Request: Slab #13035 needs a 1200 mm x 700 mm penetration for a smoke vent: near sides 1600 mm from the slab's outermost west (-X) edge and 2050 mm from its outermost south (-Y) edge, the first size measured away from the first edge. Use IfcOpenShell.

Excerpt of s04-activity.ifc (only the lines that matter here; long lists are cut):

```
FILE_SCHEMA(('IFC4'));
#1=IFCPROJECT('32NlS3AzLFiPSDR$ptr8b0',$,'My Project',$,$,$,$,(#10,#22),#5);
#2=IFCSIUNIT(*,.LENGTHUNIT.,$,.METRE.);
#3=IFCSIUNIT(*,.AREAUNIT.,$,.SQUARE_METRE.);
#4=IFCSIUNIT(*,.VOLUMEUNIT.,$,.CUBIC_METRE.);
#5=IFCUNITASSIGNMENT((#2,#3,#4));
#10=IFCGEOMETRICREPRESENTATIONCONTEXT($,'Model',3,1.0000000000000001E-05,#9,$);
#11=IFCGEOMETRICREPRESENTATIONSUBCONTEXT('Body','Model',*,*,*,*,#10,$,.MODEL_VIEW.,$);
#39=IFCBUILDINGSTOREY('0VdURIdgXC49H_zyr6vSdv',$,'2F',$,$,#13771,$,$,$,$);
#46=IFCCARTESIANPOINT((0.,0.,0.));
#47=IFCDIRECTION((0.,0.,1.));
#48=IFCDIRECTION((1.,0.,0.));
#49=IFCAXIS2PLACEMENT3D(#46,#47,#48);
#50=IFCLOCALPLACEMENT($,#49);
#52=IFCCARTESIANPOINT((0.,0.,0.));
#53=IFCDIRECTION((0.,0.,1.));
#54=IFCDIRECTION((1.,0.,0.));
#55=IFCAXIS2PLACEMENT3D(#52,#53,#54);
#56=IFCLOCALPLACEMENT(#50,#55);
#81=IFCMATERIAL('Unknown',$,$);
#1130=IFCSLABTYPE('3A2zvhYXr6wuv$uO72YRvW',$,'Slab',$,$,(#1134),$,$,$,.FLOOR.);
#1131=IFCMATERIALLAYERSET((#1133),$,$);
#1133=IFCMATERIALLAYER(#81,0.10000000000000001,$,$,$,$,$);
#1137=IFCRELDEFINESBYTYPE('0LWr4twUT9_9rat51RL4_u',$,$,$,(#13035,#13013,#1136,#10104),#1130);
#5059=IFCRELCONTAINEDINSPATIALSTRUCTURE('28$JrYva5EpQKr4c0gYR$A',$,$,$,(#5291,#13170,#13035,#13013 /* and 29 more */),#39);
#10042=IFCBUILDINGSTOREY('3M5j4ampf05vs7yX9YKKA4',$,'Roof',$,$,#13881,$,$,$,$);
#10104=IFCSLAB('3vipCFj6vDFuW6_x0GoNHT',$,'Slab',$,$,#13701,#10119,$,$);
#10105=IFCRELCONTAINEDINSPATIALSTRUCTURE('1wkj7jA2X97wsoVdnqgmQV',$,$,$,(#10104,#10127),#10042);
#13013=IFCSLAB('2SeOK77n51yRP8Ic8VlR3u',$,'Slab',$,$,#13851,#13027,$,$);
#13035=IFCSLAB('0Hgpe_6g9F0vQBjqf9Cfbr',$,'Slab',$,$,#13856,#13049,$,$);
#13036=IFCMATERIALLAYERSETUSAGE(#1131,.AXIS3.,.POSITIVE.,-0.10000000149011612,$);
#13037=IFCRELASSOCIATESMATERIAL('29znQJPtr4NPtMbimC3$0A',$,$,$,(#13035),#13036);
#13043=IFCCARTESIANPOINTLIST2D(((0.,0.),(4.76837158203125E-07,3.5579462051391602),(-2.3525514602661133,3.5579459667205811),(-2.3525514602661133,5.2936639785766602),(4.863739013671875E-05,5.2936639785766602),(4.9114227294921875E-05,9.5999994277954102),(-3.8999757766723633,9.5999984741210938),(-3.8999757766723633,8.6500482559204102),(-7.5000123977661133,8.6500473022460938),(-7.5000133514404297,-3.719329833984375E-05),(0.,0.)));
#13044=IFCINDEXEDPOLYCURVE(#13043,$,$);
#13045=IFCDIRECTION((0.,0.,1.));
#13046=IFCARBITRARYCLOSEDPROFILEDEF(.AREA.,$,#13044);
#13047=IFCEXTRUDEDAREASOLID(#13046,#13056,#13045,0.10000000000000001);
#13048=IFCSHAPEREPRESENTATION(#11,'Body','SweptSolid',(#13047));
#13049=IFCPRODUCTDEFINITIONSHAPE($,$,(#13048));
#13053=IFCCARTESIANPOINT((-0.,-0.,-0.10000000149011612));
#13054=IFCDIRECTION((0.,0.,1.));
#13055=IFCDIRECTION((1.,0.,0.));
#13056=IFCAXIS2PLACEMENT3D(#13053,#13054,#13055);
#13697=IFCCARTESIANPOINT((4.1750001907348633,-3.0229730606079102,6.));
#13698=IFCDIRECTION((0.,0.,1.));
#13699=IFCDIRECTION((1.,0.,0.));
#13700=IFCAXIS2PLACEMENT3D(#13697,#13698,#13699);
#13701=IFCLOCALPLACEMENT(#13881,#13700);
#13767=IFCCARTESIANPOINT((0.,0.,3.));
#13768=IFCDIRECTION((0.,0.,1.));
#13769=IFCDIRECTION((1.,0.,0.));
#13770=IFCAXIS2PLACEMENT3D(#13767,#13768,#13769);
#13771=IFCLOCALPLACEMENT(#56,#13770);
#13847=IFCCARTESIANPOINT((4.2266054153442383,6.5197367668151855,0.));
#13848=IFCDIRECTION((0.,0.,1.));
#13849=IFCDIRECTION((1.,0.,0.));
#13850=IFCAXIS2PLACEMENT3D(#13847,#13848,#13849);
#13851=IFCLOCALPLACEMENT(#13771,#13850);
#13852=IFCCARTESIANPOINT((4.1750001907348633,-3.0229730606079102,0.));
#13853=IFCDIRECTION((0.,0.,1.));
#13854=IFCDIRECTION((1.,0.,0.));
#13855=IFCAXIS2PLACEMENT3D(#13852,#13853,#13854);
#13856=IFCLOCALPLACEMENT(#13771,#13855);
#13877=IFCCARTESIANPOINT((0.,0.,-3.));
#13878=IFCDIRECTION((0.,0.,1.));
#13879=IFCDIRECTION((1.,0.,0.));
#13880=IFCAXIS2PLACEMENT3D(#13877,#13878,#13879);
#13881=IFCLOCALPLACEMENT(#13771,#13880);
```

```python
import numpy as np
import ifcopenshell
import ifcopenshell.api.feature
import ifcopenshell.api.geometry
import ifcopenshell.api.root
import ifcopenshell.geom
import ifcopenshell.util.placement
import ifcopenshell.util.representation
import ifcopenshell.util.shape
import ifcopenshell.util.unit

model = ifcopenshell.open("s04-activity.ifc")
unit_scale = ifcopenshell.util.unit.calculate_unit_scale(model)
settings = ifcopenshell.geom.settings()


def volume(element):
    """Net volume in cubic metres, openings subtracted."""
    shape = ifcopenshell.geom.create_shape(settings, element)
    return ifcopenshell.util.shape.get_volume(shape.geometry)


slab = model.by_id(13035)
before = volume(slab)

# Extent in the slab's own axes, in metres. The edges named are its -X and -Y sides.
slab_shape = ifcopenshell.geom.create_shape(settings, slab)
vertices = ifcopenshell.util.shape.get_vertices(slab_shape.geometry)
x_min, y_min, bottom = vertices.min(axis=0)
top = vertices[:, 2].max()

opening = ifcopenshell.api.root.create_entity(model, ifc_class="IfcOpeningElement", name="Smoke vent opening", predefined_type="OPENING")
context = ifcopenshell.util.representation.get_context(model, "Model", "Body", "MODEL_VIEW")
width, depth = 1.2, 0.7
outline = [(0.0, 0.0), (width, 0.0), (width, depth), (0.0, depth), (0.0, 0.0)]
# Overshoot both faces by 50 mm so the cut is clean.
shape = ifcopenshell.api.geometry.add_slab_representation(
    model, context=context, depth=top - bottom + 0.1, polyline=outline
)
ifcopenshell.api.geometry.assign_representation(model, product=opening, representation=shape)

matrix = ifcopenshell.util.placement.get_local_placement(slab.ObjectPlacement)
matrix[:, 3] = matrix @ np.append(np.array([x_min + 1.6, y_min + 2.05, bottom - 0.05]) / unit_scale, 1.0)
ifcopenshell.api.geometry.edit_object_placement(model, product=opening, matrix=matrix, is_si=False)
ifcopenshell.api.feature.add_feature(model, feature=opening, element=slab)

after = volume(slab)

print(f"slab volume {before:.3f} -> {after:.3f} m3")

model.write("s04-activity_edited.ifc")
```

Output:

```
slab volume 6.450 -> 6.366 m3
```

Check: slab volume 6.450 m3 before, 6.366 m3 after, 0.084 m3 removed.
